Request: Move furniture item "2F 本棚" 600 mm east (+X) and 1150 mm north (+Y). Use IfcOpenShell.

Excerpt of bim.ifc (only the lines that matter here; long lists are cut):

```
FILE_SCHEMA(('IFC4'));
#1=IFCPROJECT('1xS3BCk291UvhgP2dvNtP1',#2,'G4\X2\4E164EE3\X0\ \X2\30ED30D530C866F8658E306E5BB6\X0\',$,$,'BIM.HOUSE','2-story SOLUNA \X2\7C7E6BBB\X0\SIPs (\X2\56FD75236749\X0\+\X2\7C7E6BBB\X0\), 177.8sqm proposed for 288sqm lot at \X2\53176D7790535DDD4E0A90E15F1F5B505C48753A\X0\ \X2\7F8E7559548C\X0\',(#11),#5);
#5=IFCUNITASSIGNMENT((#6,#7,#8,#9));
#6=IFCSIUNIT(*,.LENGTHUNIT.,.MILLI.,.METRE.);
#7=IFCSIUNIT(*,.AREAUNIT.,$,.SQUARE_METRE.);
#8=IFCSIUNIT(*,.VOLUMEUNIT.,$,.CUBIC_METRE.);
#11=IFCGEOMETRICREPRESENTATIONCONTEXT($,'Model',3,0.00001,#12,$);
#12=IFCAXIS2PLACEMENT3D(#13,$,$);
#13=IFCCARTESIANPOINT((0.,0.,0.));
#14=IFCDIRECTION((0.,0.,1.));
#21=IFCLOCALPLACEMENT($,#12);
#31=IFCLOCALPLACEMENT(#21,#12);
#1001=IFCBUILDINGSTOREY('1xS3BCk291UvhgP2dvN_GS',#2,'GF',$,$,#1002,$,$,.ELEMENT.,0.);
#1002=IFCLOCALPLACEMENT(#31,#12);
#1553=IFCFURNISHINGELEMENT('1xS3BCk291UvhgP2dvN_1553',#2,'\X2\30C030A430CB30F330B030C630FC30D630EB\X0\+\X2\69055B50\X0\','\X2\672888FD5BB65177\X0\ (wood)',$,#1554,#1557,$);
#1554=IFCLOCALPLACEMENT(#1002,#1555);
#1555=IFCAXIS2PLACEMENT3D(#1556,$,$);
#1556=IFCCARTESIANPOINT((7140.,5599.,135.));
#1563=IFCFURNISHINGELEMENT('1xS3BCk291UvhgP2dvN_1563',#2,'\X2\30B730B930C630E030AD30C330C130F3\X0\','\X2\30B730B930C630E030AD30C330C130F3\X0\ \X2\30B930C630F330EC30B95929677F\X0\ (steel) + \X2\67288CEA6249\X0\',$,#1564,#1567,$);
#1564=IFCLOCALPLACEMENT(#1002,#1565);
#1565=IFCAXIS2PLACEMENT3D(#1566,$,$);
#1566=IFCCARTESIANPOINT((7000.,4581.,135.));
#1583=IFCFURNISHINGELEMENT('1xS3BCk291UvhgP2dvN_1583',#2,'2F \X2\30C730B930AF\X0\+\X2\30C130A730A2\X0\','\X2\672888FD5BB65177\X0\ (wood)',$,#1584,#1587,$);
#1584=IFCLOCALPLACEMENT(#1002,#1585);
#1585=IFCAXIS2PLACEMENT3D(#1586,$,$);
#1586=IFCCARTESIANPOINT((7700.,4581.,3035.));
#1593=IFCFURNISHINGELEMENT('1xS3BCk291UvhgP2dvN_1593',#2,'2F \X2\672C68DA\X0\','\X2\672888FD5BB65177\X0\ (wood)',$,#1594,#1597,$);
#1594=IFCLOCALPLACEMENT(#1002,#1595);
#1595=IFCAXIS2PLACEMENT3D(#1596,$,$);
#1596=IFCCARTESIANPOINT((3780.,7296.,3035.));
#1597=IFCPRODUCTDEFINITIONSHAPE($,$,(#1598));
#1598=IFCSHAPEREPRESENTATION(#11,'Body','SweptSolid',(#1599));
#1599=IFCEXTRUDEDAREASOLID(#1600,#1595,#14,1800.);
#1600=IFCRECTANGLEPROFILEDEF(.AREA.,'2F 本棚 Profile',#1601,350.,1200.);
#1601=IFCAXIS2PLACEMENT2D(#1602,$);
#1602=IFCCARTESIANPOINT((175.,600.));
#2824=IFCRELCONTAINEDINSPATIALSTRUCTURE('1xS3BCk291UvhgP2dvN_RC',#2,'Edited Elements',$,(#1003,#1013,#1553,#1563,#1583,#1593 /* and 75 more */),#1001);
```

```python
import ifcopenshell
import ifcopenshell.api.geometry
import ifcopenshell.util.placement

model = ifcopenshell.open("bim.ifc")

item = model.by_guid("1xS3BCk291UvhgP2dvN_1593")
matrix = ifcopenshell.util.placement.get_local_placement(item.ObjectPlacement)
matrix[0, 3] += 600.0
matrix[1, 3] += 1150.0
ifcopenshell.api.geometry.edit_object_placement(model, product=item, matrix=matrix, is_si=False)

print(ifcopenshell.util.placement.get_local_placement(item.ObjectPlacement).round(3) + 0.0)

model.write("bim_updated.ifc")
```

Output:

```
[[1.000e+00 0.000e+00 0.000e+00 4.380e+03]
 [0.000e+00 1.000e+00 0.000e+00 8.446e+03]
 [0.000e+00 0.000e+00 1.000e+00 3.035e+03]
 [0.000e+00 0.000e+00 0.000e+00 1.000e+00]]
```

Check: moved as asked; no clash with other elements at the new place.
